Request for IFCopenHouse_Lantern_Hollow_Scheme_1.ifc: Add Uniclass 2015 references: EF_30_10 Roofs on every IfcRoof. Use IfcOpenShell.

First a look at what the model holds.

```python
import ifcopenshell

model = ifcopenshell.open("IFCopenHouse_Lantern_Hollow_Scheme_1.ifc")
print(model.schema)
print("classifications:", [c.Name for c in model.by_type("IfcClassification")])
for ifc_class in ("IfcDoor", "IfcRoof", "IfcStair", "IfcWall", "IfcWindow"):
    print(ifc_class, len(model.by_type(ifc_class)))
```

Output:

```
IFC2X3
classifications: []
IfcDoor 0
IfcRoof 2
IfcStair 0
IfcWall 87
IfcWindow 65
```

```python
import ifcopenshell
import ifcopenshell.api.classification

model = ifcopenshell.open("IFCopenHouse_Lantern_Hollow_Scheme_1.ifc")

# IFC2X3 requires Source and Edition and has no link from the project to the system.
system = model.create_entity("IfcClassification", Source="NBS", Edition="2015", Name="Uniclass 2015")

codes = {
    "IfcRoof": ("EF_30_10", "Roofs"),
}
for ifc_class, (code, name) in codes.items():
    products = model.by_type(ifc_class)
    ifcopenshell.api.classification.add_reference(
        model, products=products, classification=system, identification=code, name=name
    )
    print(code, len(products))

model.write("IFCopenHouse_Lantern_Hollow_Scheme_1_edited.ifc")
```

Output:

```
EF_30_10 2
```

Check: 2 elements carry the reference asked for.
